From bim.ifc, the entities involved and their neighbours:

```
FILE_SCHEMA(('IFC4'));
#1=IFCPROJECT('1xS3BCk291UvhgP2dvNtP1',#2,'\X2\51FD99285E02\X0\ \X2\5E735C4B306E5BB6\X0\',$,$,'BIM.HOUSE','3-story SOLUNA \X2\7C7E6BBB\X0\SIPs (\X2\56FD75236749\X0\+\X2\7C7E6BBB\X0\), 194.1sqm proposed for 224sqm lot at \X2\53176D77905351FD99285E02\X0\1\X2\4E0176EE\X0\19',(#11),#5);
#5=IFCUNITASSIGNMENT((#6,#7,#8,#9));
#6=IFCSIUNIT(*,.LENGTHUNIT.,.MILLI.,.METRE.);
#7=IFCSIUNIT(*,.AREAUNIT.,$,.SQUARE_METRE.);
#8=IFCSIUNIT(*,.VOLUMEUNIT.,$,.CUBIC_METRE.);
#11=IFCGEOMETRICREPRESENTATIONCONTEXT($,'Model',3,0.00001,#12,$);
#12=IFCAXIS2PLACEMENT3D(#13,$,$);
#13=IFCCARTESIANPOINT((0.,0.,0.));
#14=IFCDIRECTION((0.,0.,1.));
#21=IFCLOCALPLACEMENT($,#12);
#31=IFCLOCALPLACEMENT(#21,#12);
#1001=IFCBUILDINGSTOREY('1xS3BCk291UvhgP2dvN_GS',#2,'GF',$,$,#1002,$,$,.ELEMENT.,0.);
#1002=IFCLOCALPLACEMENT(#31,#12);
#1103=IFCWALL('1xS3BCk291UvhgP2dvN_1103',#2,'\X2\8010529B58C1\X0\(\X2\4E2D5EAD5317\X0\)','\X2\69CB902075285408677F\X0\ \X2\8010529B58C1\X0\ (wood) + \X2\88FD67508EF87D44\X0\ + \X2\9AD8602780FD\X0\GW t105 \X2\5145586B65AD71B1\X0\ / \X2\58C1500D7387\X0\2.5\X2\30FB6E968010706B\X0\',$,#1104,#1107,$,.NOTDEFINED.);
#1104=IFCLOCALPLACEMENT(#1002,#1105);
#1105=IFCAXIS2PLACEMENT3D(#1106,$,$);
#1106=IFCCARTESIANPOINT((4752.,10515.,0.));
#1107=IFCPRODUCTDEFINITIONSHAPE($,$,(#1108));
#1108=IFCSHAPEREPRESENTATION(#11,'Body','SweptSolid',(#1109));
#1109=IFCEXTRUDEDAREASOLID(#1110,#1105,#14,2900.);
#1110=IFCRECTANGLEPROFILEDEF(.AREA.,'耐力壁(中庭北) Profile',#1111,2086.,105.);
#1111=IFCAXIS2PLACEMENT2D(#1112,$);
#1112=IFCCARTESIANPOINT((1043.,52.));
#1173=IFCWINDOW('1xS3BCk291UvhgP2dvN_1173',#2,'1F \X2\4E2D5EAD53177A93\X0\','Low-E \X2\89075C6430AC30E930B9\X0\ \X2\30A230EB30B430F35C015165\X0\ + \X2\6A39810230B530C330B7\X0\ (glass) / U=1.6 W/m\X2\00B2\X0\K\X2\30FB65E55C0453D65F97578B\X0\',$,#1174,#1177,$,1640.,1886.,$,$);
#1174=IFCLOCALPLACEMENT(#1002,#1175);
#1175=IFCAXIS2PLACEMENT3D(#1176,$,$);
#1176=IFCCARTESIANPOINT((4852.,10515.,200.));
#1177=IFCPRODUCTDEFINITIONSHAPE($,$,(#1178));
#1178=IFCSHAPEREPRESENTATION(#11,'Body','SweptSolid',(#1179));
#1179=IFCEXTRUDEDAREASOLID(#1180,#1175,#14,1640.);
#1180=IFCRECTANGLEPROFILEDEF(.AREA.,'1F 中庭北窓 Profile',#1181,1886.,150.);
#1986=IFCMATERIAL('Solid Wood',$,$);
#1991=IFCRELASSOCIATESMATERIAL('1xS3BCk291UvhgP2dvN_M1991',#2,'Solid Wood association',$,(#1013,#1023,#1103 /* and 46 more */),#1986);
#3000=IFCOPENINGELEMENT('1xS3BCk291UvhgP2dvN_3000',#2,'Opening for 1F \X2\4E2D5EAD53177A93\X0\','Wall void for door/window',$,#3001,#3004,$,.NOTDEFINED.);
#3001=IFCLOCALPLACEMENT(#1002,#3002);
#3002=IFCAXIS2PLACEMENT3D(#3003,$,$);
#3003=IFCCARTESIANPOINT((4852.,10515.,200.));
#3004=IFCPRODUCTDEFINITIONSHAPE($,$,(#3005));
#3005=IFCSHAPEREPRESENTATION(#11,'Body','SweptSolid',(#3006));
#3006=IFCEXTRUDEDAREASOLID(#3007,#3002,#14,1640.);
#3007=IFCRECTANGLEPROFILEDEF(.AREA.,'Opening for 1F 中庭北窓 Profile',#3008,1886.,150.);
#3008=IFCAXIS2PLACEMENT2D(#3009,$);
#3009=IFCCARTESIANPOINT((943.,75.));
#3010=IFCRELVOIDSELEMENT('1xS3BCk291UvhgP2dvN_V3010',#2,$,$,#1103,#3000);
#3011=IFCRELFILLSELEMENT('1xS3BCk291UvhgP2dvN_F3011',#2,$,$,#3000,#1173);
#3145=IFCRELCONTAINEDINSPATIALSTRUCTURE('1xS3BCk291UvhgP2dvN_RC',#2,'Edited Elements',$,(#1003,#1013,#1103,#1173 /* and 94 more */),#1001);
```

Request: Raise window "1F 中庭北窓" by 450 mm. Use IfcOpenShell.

```python
import numpy as np
import ifcopenshell
import ifcopenshell.api.geometry
import ifcopenshell.util.placement
import ifcopenshell.util.unit

model = ifcopenshell.open("bim.ifc")
unit_scale = ifcopenshell.util.unit.calculate_unit_scale(model)

window = model.by_guid("1xS3BCk291UvhgP2dvN_1173")
opening = window.FillsVoids[0].RelatingOpeningElement
dz = 450.0

shift = np.array([0.0, 0.0, dz])
# The window is not placed relative to its opening, so move both.
for product in (opening, window):
    matrix = ifcopenshell.util.placement.get_local_placement(product.ObjectPlacement)
    matrix[:3, 3] += shift
    ifcopenshell.api.geometry.edit_object_placement(model, product=product, matrix=matrix, is_si=False)

print(f"moved by {dz * unit_scale:+.3f} m")

model.write("bim_updated.ifc")
```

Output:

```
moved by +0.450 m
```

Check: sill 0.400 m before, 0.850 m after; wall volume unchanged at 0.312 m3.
